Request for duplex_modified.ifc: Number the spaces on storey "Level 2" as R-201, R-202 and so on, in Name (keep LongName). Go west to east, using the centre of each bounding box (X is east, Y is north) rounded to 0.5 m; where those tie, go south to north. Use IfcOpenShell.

First a look at what the model holds.

```python
import ifcopenshell
import ifcopenshell.util.element
import ifcopenshell.util.placement

model = ifcopenshell.open("duplex_modified.ifc")
print(model.schema)
storey = next(s for s in model.by_type("IfcBuildingStorey") if s.Name == "Level 2")
spaces = [e for e in ifcopenshell.util.element.get_decomposition(storey) if e.is_a("IfcSpace")]
for e in sorted(spaces, key=lambda e: e.id()):
    origin = ifcopenshell.util.placement.get_local_placement(e.ObjectPlacement)[:3, 3]
    print(e.id(), e.Name, e.LongName, origin.round(2) + 0.0, sep=" | ")
```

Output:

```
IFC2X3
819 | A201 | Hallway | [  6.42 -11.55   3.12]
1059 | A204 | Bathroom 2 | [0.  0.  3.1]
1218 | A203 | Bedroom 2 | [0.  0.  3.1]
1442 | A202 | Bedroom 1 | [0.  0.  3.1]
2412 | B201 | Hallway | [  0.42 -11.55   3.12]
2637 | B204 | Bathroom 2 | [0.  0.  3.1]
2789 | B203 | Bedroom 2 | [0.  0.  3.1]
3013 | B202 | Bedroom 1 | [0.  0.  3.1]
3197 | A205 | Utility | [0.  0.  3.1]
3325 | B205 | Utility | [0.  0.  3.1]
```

```python
import ifcopenshell
import ifcopenshell.geom
import ifcopenshell.util.element
import ifcopenshell.util.shape

model = ifcopenshell.open("duplex_modified.ifc")
settings = ifcopenshell.geom.settings()
settings.set("use-world-coords", True)


def centre(element):
    shape = ifcopenshell.geom.create_shape(settings, element)
    return ifcopenshell.util.shape.get_bbox_centroid(shape.geometry)


storey = next(s for s in model.by_type("IfcBuildingStorey") if s.Name == "Level 2")
spaces = [e for e in ifcopenshell.util.element.get_decomposition(storey) if e.is_a("IfcSpace")]

# Insertion points can sit at a corner or the storey origin, so sort by the geometry (in metres).
centres = {e: centre(e) for e in spaces}
spaces.sort(key=lambda e: (round(centres[e][0] / 0.5), centres[e][1]))

for i, e in enumerate(spaces, start=1):
    number = f"R-2{i:02d}"
    e.Name = number
    print(e.id(), number)

model.write("duplex_modified_updated.ifc")
```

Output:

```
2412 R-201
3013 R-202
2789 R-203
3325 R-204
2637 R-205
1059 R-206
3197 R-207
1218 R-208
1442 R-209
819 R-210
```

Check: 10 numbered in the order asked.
